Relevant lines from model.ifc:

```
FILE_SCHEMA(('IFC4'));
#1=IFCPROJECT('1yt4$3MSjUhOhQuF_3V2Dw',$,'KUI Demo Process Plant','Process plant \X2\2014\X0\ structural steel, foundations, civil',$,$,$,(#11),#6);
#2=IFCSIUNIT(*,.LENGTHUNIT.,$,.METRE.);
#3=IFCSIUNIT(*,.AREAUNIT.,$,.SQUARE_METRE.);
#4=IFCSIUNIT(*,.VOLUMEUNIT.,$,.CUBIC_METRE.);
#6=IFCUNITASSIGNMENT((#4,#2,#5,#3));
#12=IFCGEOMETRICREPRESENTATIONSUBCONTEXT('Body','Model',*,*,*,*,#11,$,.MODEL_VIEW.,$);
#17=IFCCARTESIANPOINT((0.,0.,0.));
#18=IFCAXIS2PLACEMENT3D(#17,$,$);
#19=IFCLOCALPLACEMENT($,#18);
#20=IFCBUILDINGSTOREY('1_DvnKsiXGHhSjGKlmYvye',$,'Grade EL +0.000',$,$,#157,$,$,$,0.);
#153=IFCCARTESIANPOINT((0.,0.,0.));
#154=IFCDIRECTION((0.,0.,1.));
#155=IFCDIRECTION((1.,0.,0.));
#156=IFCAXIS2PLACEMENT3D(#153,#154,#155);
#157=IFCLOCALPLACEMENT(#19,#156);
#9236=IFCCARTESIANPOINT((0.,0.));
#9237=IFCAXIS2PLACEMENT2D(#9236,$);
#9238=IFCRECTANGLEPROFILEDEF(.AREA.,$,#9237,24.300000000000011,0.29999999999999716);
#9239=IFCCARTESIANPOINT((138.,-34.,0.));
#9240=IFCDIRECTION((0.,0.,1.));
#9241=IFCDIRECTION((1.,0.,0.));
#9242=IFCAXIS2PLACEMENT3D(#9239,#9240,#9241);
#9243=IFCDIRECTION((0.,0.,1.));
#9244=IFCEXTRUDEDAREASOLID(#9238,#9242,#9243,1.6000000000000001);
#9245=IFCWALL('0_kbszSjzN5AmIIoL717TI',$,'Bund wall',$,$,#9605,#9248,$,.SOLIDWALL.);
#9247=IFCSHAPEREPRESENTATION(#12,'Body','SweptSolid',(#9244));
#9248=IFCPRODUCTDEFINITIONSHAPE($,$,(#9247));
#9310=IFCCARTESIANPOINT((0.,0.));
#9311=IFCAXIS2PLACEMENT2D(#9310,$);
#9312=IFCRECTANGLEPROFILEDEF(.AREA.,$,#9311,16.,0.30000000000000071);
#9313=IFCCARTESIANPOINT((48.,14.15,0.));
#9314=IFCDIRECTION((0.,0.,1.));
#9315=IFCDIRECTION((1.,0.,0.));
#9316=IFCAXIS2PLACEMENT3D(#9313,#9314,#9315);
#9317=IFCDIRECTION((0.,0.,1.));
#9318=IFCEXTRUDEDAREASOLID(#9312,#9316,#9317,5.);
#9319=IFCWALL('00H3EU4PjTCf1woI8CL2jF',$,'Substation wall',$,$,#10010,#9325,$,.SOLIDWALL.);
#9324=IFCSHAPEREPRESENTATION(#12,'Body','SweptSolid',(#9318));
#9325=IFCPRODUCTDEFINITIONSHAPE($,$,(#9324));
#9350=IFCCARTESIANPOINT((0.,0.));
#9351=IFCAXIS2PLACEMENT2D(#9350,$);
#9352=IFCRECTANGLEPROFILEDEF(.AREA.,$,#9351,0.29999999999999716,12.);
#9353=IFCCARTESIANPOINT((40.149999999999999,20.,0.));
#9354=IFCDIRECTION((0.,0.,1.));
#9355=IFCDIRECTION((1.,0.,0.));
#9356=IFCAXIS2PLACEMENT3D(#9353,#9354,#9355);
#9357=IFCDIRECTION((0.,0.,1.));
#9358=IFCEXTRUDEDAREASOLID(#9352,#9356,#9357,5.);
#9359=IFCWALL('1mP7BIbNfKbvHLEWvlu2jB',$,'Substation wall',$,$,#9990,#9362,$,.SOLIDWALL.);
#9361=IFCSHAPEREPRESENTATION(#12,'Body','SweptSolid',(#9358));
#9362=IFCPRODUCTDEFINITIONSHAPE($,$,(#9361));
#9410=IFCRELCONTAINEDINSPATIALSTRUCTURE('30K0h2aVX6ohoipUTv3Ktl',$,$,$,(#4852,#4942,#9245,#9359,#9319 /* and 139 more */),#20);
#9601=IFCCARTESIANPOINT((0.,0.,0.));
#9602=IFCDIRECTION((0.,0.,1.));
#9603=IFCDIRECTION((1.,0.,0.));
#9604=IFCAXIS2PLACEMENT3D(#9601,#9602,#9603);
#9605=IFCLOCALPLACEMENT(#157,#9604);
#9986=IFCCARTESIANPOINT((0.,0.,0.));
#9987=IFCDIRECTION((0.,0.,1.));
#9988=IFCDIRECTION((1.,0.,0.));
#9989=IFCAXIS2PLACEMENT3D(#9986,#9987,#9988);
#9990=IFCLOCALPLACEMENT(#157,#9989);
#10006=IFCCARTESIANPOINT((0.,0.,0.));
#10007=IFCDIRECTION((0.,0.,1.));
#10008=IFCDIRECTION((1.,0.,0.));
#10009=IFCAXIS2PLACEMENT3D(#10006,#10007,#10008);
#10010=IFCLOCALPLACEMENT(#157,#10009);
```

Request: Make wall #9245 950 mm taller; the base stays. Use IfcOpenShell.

```python
import ifcopenshell
import ifcopenshell.geom
import ifcopenshell.util.representation
import ifcopenshell.util.shape
import ifcopenshell.util.unit

model = ifcopenshell.open("model.ifc")
unit_scale = ifcopenshell.util.unit.calculate_unit_scale(model)
settings = ifcopenshell.geom.settings()


def volume(element):
    """Net volume in cubic metres, openings subtracted."""
    shape = ifcopenshell.geom.create_shape(settings, element)
    return ifcopenshell.util.shape.get_volume(shape.geometry)


wall = model.by_id(9245)
before = volume(wall)

body = ifcopenshell.util.representation.get_representation(wall, "Model", "Body")
solid = body.Items[0]
old_height = solid.Depth
solid.Depth += 0.95 / unit_scale
after = volume(wall)

print(f"height {old_height:g} -> {solid.Depth:g}, volume {before:.3f} -> {after:.3f} m3")

model.write("model_v2.ifc")
```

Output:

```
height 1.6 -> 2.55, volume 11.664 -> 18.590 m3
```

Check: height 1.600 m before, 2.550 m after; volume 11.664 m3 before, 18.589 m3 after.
